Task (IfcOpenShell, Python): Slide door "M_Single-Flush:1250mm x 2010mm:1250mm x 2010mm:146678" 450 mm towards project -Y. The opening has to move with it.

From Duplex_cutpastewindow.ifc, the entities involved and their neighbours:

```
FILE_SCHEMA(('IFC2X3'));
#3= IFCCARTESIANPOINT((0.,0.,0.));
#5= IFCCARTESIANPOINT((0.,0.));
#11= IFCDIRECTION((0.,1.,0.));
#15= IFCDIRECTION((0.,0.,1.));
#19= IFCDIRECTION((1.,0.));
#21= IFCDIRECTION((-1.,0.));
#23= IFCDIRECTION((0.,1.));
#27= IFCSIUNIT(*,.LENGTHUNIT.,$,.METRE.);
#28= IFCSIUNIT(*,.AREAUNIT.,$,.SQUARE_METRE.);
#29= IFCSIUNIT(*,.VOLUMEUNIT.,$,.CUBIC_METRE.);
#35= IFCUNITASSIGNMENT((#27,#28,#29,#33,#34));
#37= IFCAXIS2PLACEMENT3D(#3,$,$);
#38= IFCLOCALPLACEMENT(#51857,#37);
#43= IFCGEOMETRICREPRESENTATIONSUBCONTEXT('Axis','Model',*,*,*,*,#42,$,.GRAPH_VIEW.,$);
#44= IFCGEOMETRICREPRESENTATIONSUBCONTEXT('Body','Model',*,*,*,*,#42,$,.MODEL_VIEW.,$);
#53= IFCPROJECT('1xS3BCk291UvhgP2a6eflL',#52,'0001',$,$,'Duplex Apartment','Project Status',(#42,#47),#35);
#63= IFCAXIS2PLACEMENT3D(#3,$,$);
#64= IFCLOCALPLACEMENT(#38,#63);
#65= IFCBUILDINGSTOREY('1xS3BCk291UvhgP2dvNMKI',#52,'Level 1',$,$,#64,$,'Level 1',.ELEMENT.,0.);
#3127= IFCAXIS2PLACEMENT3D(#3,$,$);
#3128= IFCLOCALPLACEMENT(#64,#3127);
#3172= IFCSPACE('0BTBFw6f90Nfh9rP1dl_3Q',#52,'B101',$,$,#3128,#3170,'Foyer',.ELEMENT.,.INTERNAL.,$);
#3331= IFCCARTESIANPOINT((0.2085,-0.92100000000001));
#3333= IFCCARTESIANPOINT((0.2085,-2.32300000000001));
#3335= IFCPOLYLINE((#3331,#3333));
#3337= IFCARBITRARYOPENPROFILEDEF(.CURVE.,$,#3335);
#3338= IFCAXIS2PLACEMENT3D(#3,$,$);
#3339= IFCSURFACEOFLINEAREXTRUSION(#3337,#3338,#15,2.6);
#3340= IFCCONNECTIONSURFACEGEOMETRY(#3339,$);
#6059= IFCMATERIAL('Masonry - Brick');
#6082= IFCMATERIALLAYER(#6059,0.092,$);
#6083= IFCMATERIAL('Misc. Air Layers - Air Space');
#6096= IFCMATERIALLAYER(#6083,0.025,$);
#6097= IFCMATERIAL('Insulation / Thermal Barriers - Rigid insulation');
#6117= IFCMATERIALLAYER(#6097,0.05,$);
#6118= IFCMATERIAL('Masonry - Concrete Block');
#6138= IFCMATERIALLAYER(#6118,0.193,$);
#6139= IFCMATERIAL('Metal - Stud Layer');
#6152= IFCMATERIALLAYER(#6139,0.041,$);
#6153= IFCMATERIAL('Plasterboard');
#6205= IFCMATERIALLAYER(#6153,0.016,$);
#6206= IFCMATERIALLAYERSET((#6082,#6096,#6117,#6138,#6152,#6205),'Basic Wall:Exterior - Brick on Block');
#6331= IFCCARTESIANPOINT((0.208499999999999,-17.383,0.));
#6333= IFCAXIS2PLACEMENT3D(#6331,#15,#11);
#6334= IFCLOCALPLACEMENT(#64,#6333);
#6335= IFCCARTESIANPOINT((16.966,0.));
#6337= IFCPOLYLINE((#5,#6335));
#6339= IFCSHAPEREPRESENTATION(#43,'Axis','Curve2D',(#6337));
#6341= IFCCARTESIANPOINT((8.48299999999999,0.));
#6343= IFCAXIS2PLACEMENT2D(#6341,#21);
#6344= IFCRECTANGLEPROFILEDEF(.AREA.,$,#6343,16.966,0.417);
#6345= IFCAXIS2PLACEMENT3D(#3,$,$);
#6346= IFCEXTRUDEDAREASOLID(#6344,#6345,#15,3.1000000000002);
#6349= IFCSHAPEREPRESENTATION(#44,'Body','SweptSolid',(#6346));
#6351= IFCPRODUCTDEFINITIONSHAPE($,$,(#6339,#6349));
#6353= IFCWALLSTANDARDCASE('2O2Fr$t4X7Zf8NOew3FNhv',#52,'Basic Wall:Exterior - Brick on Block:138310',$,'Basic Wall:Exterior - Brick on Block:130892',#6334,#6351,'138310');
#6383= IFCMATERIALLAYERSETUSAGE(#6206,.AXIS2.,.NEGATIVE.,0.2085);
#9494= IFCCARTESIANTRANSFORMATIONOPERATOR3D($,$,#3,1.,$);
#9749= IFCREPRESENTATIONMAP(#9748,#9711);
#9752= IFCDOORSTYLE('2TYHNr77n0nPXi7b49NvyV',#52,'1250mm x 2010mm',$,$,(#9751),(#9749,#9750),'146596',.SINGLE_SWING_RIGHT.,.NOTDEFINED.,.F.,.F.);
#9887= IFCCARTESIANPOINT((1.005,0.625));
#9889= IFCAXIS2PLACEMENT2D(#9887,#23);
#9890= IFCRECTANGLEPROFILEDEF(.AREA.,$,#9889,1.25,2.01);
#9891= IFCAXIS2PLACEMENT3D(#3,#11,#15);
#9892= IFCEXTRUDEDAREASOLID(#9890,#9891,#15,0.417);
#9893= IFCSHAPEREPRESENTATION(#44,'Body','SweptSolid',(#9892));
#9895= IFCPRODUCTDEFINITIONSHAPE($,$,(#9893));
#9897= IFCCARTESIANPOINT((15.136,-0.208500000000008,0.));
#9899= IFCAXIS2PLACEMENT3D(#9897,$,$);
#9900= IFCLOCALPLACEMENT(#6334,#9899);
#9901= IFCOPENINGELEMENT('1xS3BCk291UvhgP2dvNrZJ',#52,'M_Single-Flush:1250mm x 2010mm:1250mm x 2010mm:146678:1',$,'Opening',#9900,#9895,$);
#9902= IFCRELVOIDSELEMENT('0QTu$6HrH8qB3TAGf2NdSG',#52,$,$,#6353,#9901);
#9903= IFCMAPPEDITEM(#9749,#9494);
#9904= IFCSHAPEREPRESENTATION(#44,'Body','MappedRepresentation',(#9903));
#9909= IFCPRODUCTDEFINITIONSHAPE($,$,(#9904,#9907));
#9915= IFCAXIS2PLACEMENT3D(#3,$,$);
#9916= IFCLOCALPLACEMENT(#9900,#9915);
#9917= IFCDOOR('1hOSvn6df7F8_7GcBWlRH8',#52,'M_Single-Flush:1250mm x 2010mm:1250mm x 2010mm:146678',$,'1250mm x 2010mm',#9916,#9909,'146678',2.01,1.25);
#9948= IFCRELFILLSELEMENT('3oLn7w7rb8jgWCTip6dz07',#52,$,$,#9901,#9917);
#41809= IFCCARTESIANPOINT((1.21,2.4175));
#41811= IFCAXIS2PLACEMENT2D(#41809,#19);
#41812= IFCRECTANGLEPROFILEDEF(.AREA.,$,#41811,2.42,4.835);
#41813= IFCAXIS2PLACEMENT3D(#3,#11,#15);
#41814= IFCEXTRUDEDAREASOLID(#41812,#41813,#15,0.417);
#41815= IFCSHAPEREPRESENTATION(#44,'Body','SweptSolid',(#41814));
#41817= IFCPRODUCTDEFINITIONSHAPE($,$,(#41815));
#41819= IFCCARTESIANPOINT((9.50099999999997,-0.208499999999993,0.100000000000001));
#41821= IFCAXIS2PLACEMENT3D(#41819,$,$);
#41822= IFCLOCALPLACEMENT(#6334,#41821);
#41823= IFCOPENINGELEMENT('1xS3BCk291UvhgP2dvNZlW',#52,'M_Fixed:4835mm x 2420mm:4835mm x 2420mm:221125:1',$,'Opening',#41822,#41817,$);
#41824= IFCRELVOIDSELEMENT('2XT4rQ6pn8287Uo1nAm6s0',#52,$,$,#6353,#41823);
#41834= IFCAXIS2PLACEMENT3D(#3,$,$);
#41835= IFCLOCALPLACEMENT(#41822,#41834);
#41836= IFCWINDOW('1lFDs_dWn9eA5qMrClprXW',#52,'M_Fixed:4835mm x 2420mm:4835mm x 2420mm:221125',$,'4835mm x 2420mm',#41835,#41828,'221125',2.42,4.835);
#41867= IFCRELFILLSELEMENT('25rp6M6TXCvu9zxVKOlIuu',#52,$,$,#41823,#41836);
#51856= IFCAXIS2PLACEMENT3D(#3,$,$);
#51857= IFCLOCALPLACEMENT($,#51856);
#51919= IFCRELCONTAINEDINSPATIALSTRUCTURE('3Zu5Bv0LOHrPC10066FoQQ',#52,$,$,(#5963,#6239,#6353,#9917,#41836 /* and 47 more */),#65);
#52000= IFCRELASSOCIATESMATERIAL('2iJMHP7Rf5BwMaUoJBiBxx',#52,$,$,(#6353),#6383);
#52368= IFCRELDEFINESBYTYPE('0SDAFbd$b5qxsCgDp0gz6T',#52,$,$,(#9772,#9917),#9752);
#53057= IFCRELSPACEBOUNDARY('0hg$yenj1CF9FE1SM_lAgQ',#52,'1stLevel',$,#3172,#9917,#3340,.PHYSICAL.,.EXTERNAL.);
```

```python
import numpy as np
import ifcopenshell
import ifcopenshell.api.geometry
import ifcopenshell.util.placement

model = ifcopenshell.open("Duplex_cutpastewindow.ifc")

door = model.by_guid("1hOSvn6df7F8_7GcBWlRH8")
opening = door.FillsVoids[0].RelatingOpeningElement
wall = opening.VoidsElements[0].RelatingBuildingElement

wall_matrix = ifcopenshell.util.placement.get_local_placement(wall.ObjectPlacement)
shift = wall_matrix[:3, 0] * -0.45
before = ifcopenshell.util.placement.get_local_placement(door.ObjectPlacement)[:3, 3].copy()

# The door is placed relative to its opening, so it follows when the opening moves.
matrix = ifcopenshell.util.placement.get_local_placement(opening.ObjectPlacement)
matrix[:3, 3] += shift
ifcopenshell.api.geometry.edit_object_placement(
    model, product=opening, matrix=matrix, is_si=False, should_transform_children=True
)

# Space boundary surfaces are stored in each space's coordinates; move them too.
for rel in door.ProvidesBoundaries:
    if not rel.ConnectionGeometry:
        continue
    surface = rel.ConnectionGeometry.SurfaceOnRelatingElement
    space_matrix = ifcopenshell.util.placement.get_local_placement(rel.RelatingSpace.ObjectPlacement)
    point = np.array(surface.Position.Location.Coordinates) + space_matrix[:3, :3].T @ shift
    surface.Position = model.createIfcAxis2Placement3D(
        model.createIfcCartesianPoint(point.tolist()), surface.Position.Axis, surface.Position.RefDirection
    )

after = ifcopenshell.util.placement.get_local_placement(door.ObjectPlacement)[:3, 3]
print("door moved by", (after - before).round(3) + 0.0)

model.write("Duplex_cutpastewindow_v2.ifc")
```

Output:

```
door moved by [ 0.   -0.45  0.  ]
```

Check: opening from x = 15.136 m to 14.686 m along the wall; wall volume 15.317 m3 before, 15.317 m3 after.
